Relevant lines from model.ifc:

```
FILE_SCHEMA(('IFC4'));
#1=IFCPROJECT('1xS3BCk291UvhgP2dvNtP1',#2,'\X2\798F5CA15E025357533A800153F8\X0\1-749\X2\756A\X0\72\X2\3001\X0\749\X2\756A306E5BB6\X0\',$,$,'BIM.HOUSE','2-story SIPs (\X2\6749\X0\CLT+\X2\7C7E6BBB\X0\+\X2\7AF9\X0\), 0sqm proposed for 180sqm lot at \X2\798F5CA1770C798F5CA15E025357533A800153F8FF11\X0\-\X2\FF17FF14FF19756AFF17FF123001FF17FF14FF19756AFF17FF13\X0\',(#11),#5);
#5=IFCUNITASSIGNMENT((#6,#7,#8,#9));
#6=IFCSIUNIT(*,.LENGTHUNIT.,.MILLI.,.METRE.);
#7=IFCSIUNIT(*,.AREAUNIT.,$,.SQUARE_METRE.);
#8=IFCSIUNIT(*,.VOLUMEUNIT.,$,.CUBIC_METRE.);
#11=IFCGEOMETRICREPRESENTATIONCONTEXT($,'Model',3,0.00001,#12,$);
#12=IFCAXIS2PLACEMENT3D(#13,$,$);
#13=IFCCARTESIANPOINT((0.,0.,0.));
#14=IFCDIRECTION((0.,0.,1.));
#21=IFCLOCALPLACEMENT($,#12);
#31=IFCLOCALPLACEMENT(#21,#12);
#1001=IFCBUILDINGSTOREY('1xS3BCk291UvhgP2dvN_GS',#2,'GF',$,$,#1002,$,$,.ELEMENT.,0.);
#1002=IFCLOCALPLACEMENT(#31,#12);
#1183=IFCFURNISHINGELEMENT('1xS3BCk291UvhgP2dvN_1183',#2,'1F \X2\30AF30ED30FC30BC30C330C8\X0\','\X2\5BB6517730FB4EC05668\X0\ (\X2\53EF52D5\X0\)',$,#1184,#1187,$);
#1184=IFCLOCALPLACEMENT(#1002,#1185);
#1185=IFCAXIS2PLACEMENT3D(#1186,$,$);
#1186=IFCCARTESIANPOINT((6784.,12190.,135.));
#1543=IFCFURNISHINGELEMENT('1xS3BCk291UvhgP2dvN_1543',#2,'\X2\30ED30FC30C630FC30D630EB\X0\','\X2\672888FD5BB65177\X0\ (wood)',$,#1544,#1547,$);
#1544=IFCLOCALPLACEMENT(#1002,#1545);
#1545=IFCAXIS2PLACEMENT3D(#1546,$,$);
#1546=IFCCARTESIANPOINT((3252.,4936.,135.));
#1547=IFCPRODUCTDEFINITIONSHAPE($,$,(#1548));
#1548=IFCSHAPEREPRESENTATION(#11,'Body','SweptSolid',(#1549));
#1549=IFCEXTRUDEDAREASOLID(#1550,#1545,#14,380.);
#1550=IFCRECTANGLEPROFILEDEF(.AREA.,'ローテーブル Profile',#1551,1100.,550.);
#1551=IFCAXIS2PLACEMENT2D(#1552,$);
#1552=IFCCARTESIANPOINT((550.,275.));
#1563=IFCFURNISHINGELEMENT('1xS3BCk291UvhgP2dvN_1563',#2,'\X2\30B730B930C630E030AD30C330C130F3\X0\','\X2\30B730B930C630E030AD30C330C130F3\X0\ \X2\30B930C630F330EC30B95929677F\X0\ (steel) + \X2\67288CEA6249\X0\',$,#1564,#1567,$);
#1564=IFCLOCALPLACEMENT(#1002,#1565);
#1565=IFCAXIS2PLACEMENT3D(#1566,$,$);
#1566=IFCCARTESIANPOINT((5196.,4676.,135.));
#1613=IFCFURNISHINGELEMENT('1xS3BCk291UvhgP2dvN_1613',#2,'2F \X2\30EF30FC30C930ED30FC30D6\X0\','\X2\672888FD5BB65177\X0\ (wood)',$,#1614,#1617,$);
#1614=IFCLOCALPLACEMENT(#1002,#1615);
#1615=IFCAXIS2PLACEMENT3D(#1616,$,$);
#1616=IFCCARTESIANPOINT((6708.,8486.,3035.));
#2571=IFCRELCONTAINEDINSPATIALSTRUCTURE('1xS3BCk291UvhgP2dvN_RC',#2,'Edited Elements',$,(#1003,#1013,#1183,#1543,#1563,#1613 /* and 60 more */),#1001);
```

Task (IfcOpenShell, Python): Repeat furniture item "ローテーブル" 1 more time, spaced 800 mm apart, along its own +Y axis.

```python
import ifcopenshell
import ifcopenshell.api.geometry
import ifcopenshell.api.root
import ifcopenshell.util.element
import ifcopenshell.util.placement
import ifcopenshell.util.unit

model = ifcopenshell.open("model.ifc")
unit_scale = ifcopenshell.util.unit.calculate_unit_scale(model)


def reuse_history(source, copy):
    """copy_class also copies each property set's owner history, people and application; keep the originals."""
    for rel in copy.IsDefinedBy:
        if rel.is_a("IfcRelDefinesByProperties") and (history := rel.RelatingPropertyDefinition.OwnerHistory):
            rel.RelatingPropertyDefinition.OwnerHistory = source.OwnerHistory
            ifcopenshell.util.element.remove_deep2(model, history)


source = model.by_guid("1xS3BCk291UvhgP2dvN_1543")
base = ifcopenshell.util.placement.get_local_placement(source.ObjectPlacement)
step = base[:3, 1] * 0.8 / unit_scale

for i in range(1, 2):
    copy = ifcopenshell.api.root.copy_class(model, product=source)
    copy.Representation = ifcopenshell.util.element.copy_deep(
        model, source.Representation, exclude=["IfcGeometricRepresentationContext", "IfcRepresentationMap"]
    )
    reuse_history(source, copy)
    matrix = base.copy()
    matrix[:3, 3] += i * step
    print("added at", matrix[:3, 3].round(3) + 0.0)
    ifcopenshell.api.geometry.edit_object_placement(model, product=copy, matrix=matrix, is_si=False)

model.write("model_updated.ifc")
```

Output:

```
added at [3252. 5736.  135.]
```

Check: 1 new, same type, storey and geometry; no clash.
